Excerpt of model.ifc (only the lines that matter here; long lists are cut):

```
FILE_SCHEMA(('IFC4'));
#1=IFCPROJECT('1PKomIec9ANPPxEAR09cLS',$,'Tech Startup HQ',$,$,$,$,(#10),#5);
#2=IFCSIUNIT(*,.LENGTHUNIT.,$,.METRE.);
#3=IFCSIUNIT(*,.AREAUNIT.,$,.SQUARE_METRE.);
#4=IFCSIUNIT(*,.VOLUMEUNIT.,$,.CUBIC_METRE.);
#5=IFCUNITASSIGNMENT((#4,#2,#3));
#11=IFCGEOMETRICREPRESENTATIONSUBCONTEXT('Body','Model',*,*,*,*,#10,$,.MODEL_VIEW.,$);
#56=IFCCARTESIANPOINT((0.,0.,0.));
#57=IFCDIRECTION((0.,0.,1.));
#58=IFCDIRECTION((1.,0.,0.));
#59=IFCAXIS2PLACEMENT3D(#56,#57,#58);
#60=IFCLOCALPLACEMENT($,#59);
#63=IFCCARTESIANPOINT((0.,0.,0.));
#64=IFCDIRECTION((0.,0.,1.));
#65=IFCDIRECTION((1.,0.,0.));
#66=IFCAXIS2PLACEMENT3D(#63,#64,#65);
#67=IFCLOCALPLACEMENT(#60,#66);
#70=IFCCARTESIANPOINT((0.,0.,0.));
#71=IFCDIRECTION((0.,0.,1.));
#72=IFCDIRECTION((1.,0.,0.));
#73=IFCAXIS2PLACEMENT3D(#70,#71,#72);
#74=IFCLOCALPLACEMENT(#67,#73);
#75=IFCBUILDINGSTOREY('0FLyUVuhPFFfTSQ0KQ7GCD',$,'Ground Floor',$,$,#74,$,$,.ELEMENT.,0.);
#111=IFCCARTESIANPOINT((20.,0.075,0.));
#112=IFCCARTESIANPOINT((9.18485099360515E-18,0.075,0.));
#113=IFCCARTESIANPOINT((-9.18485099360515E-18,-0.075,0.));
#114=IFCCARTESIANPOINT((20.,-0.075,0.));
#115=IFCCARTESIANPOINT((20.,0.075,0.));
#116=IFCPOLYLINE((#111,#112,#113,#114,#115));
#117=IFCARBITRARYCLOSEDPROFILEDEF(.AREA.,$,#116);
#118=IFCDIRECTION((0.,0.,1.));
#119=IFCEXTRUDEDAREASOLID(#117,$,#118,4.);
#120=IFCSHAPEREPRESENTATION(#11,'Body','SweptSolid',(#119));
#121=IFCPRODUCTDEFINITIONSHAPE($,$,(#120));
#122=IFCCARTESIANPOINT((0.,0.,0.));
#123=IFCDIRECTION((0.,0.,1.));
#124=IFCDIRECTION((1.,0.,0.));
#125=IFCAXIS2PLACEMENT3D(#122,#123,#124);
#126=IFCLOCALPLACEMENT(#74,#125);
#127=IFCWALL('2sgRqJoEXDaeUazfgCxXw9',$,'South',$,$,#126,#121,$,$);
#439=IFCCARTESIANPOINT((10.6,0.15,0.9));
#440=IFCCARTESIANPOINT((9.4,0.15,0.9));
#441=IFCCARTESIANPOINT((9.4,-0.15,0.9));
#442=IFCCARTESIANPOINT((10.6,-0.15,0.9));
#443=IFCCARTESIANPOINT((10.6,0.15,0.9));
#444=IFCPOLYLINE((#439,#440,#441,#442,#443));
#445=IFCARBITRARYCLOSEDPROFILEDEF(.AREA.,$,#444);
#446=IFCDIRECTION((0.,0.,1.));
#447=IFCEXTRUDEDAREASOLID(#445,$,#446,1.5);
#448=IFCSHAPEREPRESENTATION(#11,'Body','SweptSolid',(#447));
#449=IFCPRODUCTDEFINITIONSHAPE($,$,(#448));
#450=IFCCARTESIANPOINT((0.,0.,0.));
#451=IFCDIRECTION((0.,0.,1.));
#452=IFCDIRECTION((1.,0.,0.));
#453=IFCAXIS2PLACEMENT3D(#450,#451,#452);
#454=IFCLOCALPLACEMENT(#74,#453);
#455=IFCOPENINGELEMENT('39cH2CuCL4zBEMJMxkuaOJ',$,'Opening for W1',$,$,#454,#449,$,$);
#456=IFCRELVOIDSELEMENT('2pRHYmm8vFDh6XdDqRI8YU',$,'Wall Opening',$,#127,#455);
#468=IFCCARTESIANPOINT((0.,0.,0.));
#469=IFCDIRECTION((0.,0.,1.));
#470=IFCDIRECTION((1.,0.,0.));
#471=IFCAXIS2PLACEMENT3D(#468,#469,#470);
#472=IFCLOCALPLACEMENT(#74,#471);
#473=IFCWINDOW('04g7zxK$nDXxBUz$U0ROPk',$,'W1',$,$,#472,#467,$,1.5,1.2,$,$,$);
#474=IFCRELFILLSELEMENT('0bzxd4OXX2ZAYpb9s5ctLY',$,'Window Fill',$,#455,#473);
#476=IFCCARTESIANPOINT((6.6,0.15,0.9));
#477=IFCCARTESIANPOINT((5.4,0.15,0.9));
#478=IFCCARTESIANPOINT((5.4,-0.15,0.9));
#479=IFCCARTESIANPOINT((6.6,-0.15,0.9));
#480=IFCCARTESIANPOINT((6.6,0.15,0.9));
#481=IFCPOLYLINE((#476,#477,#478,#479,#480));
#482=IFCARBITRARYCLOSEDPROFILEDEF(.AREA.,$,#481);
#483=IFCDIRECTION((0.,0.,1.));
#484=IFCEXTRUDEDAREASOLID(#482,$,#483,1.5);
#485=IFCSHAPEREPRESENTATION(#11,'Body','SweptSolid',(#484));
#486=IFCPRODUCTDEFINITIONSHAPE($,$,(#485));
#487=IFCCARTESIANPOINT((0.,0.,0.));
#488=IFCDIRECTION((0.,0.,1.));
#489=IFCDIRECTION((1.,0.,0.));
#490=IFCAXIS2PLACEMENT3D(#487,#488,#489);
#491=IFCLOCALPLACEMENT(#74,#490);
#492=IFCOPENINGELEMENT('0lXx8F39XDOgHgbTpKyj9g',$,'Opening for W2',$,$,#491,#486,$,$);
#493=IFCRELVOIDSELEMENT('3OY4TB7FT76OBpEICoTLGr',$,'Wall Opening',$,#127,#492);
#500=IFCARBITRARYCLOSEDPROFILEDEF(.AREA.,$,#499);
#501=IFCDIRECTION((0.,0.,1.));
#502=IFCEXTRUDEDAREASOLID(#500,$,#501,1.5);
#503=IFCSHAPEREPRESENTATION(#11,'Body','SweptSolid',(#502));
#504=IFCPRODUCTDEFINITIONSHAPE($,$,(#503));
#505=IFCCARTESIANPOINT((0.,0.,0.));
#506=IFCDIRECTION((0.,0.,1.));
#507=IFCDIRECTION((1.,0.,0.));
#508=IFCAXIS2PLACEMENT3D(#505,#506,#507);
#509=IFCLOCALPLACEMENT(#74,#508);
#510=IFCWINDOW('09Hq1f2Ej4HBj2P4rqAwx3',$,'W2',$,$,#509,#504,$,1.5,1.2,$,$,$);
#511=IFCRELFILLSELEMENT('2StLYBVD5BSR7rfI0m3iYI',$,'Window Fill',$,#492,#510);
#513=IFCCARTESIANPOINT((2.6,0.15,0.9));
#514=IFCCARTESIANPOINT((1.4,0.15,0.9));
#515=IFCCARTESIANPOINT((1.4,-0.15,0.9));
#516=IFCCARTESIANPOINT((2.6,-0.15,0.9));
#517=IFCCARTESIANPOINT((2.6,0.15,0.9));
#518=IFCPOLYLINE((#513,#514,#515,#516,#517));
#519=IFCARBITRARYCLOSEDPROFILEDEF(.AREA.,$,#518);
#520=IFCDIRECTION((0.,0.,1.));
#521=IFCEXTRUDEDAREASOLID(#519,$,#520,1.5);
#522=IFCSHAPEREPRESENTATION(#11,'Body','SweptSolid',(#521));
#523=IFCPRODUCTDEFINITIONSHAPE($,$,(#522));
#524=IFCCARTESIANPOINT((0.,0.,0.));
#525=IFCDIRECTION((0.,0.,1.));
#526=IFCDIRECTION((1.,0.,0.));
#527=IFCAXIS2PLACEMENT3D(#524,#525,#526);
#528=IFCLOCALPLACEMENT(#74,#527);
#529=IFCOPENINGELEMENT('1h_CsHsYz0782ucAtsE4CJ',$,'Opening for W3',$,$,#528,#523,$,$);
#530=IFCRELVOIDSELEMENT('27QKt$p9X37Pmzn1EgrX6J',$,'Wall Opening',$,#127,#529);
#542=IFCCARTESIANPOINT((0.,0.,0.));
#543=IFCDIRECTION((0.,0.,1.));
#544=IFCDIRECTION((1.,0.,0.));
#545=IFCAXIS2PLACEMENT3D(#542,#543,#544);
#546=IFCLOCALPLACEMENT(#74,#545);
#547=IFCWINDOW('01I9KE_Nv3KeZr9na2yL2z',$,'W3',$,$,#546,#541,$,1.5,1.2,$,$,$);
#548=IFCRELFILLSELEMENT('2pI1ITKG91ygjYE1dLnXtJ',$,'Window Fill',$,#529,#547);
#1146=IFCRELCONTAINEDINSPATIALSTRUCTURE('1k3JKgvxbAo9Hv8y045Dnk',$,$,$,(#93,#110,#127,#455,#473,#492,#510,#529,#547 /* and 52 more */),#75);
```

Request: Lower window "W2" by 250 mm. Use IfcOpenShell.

```python
import numpy as np
import ifcopenshell
import ifcopenshell.api.geometry
import ifcopenshell.util.placement
import ifcopenshell.util.unit

model = ifcopenshell.open("model.ifc")
unit_scale = ifcopenshell.util.unit.calculate_unit_scale(model)

window = model.by_id(510)
opening = window.FillsVoids[0].RelatingOpeningElement
dz = -0.25 / unit_scale

shift = np.array([0.0, 0.0, dz])
# The window is not placed relative to its opening, so move both.
for product in (opening, window):
    matrix = ifcopenshell.util.placement.get_local_placement(product.ObjectPlacement)
    matrix[:3, 3] += shift
    ifcopenshell.api.geometry.edit_object_placement(model, product=product, matrix=matrix, is_si=False)

print(f"moved by {dz * unit_scale:+.3f} m")

model.write("model-out.ifc")
```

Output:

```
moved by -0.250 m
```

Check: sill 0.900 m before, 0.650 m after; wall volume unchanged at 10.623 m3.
